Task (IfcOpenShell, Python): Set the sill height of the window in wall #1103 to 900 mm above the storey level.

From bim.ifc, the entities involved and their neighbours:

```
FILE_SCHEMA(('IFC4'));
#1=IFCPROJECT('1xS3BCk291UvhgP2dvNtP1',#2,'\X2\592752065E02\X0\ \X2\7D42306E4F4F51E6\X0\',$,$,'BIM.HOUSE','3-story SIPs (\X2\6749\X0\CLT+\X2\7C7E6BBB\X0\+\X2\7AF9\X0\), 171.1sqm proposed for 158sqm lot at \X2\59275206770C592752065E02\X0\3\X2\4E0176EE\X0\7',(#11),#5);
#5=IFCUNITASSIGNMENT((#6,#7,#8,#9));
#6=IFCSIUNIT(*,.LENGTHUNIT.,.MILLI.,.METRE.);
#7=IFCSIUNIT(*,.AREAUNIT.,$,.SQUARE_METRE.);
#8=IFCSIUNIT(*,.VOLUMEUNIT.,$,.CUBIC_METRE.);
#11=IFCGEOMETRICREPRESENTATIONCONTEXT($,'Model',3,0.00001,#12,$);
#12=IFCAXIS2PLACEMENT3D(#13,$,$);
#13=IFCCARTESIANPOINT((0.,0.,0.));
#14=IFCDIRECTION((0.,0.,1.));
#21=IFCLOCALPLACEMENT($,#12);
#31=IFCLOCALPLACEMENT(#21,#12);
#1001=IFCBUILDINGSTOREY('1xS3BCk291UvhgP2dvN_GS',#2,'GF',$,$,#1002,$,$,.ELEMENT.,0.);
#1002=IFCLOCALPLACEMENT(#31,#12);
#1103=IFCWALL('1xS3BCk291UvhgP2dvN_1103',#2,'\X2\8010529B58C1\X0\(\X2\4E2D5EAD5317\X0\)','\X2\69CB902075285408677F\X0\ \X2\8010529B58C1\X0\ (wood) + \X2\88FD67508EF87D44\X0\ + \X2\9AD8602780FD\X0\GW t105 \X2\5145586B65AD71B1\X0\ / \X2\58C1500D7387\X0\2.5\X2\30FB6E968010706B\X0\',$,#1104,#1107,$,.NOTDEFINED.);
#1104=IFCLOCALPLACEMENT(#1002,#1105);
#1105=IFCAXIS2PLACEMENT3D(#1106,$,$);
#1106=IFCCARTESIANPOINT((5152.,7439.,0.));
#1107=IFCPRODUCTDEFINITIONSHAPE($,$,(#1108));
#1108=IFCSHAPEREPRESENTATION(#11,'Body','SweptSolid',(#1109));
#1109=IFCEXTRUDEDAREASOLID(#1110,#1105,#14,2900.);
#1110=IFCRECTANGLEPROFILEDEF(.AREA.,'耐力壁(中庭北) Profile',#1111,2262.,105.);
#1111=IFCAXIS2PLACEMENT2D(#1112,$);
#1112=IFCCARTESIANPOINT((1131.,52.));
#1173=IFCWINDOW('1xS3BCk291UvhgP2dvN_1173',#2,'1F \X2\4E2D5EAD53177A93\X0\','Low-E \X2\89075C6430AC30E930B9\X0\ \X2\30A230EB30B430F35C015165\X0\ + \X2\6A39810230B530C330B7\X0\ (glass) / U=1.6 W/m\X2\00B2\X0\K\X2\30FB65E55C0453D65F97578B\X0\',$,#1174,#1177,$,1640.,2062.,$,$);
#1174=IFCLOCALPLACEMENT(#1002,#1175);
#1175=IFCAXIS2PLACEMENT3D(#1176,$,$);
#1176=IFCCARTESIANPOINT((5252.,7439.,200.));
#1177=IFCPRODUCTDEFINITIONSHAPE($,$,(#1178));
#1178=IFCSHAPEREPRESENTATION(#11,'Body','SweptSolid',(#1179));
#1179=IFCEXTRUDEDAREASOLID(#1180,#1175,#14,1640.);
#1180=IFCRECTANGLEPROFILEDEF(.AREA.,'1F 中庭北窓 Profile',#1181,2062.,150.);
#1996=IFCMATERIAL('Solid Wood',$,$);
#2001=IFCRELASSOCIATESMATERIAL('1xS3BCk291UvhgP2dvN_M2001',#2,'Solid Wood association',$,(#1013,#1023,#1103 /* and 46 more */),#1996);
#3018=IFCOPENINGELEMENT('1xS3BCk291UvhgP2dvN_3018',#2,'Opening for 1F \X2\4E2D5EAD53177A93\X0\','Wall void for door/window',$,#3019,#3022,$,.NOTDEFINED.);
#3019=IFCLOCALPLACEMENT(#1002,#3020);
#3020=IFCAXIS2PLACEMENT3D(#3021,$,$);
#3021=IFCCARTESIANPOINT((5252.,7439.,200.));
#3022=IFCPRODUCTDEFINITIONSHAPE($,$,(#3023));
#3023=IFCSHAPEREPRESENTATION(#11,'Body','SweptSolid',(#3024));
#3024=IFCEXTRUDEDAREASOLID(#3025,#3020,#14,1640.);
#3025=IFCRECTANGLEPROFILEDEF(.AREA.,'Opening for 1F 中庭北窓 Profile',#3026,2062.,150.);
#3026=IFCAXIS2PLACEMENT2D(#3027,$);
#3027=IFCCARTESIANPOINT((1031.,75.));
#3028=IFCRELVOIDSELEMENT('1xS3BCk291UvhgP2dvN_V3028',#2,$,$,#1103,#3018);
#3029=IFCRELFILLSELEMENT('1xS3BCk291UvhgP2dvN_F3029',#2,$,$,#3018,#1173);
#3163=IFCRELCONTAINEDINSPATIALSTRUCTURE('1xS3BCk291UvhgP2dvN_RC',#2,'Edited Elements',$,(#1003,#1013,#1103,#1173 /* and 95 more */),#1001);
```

```python
import numpy as np
import ifcopenshell
import ifcopenshell.api.geometry
import ifcopenshell.geom
import ifcopenshell.util.element
import ifcopenshell.util.placement
import ifcopenshell.util.shape
import ifcopenshell.util.unit

model = ifcopenshell.open("bim.ifc")
unit_scale = ifcopenshell.util.unit.calculate_unit_scale(model)

window = model.by_id(1173)
opening = window.FillsVoids[0].RelatingOpeningElement
storey = ifcopenshell.util.element.get_container(window, ifc_class="IfcBuildingStorey")
level = ifcopenshell.util.placement.get_local_placement(storey.ObjectPlacement)[2, 3]

# The opening's origin need not be at the sill, so measure its lowest point.
shape = ifcopenshell.geom.create_shape(ifcopenshell.geom.settings(), opening)
bottom = ifcopenshell.util.shape.get_shape_bottom_elevation(shape, shape.geometry) / unit_scale
dz = level + 900.0 - bottom

shift = np.array([0.0, 0.0, dz])
# The window is not placed relative to its opening, so move both.
for product in (opening, window):
    matrix = ifcopenshell.util.placement.get_local_placement(product.ObjectPlacement)
    matrix[:3, 3] += shift
    ifcopenshell.api.geometry.edit_object_placement(model, product=product, matrix=matrix, is_si=False)

print(f"moved by {dz * unit_scale:+.3f} m")

model.write("bim_v2.ifc")
```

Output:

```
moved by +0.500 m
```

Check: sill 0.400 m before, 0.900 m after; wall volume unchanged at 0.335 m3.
